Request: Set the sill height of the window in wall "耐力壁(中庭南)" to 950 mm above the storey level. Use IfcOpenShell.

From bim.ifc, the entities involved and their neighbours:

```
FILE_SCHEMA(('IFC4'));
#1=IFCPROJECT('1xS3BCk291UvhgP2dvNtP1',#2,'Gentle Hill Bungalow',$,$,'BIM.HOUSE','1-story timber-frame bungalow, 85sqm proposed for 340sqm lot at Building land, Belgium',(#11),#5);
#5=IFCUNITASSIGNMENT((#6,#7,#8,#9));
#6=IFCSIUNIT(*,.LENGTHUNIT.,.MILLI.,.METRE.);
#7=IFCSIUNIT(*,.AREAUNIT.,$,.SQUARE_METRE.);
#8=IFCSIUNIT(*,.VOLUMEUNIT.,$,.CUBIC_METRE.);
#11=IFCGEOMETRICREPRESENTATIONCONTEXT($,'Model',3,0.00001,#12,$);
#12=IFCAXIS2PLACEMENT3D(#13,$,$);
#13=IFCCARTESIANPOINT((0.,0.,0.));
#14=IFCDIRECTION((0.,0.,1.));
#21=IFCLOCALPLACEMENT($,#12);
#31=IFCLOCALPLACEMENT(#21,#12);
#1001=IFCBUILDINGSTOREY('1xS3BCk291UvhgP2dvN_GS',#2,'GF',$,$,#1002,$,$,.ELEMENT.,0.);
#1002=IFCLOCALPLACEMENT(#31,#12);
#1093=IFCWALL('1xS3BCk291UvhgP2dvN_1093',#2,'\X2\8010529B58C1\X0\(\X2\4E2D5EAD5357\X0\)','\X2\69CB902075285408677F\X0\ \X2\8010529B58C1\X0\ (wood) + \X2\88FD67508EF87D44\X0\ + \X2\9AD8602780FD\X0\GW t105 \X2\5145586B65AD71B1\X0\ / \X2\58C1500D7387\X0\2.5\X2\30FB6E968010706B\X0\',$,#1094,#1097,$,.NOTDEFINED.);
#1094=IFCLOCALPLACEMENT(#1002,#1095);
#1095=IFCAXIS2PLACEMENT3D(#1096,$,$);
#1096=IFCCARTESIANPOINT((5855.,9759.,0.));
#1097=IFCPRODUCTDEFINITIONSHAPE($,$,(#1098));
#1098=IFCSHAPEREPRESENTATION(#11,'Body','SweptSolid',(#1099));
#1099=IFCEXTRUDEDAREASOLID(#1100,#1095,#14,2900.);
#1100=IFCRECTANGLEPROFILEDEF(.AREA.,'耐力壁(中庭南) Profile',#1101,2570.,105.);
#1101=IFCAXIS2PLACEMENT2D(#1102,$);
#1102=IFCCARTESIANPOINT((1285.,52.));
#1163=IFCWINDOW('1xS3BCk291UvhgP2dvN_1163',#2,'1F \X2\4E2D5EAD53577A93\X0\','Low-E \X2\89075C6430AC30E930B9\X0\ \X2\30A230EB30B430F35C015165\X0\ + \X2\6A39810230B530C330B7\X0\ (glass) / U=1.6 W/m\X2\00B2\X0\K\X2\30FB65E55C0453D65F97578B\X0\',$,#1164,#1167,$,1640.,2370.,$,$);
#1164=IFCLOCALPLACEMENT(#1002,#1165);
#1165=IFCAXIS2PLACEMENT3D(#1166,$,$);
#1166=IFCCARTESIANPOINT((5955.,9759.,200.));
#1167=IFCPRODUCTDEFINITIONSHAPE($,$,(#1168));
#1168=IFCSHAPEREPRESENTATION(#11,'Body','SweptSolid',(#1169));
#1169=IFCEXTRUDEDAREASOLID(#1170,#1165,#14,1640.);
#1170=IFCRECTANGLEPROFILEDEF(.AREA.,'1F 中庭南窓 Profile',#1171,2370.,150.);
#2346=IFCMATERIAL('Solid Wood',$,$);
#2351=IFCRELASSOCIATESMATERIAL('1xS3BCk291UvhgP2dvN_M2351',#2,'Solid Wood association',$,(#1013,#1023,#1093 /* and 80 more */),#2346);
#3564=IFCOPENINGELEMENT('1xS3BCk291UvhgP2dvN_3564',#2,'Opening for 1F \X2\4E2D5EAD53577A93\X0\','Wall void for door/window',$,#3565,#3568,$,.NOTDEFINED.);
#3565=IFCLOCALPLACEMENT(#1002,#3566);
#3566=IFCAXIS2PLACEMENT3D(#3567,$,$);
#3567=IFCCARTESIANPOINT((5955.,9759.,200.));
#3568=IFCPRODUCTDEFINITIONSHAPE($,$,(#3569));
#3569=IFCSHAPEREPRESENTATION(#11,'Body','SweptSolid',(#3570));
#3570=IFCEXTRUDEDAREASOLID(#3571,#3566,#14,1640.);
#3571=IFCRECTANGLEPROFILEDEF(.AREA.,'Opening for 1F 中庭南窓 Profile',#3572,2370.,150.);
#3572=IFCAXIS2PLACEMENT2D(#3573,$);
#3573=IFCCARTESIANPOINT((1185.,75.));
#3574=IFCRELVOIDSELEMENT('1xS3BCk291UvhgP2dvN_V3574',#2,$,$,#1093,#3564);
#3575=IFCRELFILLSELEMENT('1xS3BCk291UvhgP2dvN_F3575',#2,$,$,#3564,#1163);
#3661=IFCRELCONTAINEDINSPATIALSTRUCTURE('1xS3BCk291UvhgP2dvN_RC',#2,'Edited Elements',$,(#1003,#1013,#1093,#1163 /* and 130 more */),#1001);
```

```python
import numpy as np
import ifcopenshell
import ifcopenshell.api.geometry
import ifcopenshell.geom
import ifcopenshell.util.element
import ifcopenshell.util.placement
import ifcopenshell.util.shape
import ifcopenshell.util.unit

model = ifcopenshell.open("bim.ifc")
unit_scale = ifcopenshell.util.unit.calculate_unit_scale(model)

window = model.by_guid("1xS3BCk291UvhgP2dvN_1163")
opening = window.FillsVoids[0].RelatingOpeningElement
storey = ifcopenshell.util.element.get_container(window, ifc_class="IfcBuildingStorey")
level = ifcopenshell.util.placement.get_local_placement(storey.ObjectPlacement)[2, 3]

# The opening's origin need not be at the sill, so measure its lowest point.
shape = ifcopenshell.geom.create_shape(ifcopenshell.geom.settings(), opening)
bottom = ifcopenshell.util.shape.get_shape_bottom_elevation(shape, shape.geometry) / unit_scale
dz = level + 0.95 / unit_scale - bottom

shift = np.array([0.0, 0.0, dz])
# The window is not placed relative to its opening, so move both.
for product in (opening, window):
    matrix = ifcopenshell.util.placement.get_local_placement(product.ObjectPlacement)
    matrix[:3, 3] += shift
    ifcopenshell.api.geometry.edit_object_placement(model, product=product, matrix=matrix, is_si=False)

print(f"moved by {dz * unit_scale:+.3f} m")

model.write("bim_edited.ifc")
```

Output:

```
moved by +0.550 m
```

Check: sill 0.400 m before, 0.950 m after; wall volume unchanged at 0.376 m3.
